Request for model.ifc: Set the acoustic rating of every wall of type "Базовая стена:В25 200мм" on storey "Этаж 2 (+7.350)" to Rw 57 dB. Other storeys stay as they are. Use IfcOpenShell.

First a look at what the model holds.

```python
import ifcopenshell
import ifcopenshell.util.element

model = ifcopenshell.open("model.ifc")
print(model.schema)
storey = next(s for s in model.by_type("IfcBuildingStorey") if s.Name == "Этаж 2 (+7.350)")
walls = [e for e in ifcopenshell.util.element.get_decomposition(storey) if e.is_a("IfcWall")]
seen = {}
for e in walls:
    element_type = ifcopenshell.util.element.get_type(e)
    key = (element_type.Name if element_type != e and element_type else None, ifcopenshell.util.element.get_pset(e, "Pset_WallCommon", "AcousticRating"))
    seen[key] = seen.get(key, 0) + 1
for (name, value), count in sorted(seen.items(), key=str):
    print(count, "x", name, "|", value)
```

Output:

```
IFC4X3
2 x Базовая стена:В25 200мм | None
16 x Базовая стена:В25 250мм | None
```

```python
import ifcopenshell
import ifcopenshell.api.pset
import ifcopenshell.util.element

model = ifcopenshell.open("model.ifc")

storey = next(s for s in model.by_type("IfcBuildingStorey") if s.Name == "Этаж 2 (+7.350)")
walls = [e for e in ifcopenshell.util.element.get_decomposition(storey) if e.is_a("IfcWall")]

count = 0
for e in walls:
    element_type = ifcopenshell.util.element.get_type(e)
    if element_type in (None, e) or element_type.Name != "Базовая стена:В25 200мм":
        continue
    # add_pset returns the element's existing set when there is one.
    pset = ifcopenshell.api.pset.add_pset(model, product=e, name="Pset_WallCommon")
    ifcopenshell.api.pset.edit_pset(model, pset=pset, properties={"AcousticRating": "Rw 57 dB"})
    count += 1

print(count, "walls updated")

model.write("model_v2.ifc")
```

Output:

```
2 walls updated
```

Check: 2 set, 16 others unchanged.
